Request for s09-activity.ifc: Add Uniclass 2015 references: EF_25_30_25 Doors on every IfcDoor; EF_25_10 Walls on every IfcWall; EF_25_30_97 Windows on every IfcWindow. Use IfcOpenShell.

First a look at what the model holds.

```python
import ifcopenshell

model = ifcopenshell.open("s09-activity.ifc")
print(model.schema)
print("classifications:", [c.Name for c in model.by_type("IfcClassification")])
for ifc_class in ("IfcDoor", "IfcRoof", "IfcStair", "IfcWall", "IfcWindow"):
    print(ifc_class, len(model.by_type(ifc_class)))
```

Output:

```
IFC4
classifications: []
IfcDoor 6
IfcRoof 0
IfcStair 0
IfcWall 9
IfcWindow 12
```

```python
import ifcopenshell
import ifcopenshell.api.classification

model = ifcopenshell.open("s09-activity.ifc")

system = ifcopenshell.api.classification.add_classification(model, classification="Uniclass 2015")

codes = {
    "IfcDoor": ("EF_25_30_25", "Doors"),
    "IfcWall": ("EF_25_10", "Walls"),
    "IfcWindow": ("EF_25_30_97", "Windows"),
}
for ifc_class, (code, name) in codes.items():
    products = model.by_type(ifc_class)
    ifcopenshell.api.classification.add_reference(
        model, products=products, classification=system, identification=code, name=name
    )
    print(code, len(products))

model.write("s09-activity-out.ifc")
```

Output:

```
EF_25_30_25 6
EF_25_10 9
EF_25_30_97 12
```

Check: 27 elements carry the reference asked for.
